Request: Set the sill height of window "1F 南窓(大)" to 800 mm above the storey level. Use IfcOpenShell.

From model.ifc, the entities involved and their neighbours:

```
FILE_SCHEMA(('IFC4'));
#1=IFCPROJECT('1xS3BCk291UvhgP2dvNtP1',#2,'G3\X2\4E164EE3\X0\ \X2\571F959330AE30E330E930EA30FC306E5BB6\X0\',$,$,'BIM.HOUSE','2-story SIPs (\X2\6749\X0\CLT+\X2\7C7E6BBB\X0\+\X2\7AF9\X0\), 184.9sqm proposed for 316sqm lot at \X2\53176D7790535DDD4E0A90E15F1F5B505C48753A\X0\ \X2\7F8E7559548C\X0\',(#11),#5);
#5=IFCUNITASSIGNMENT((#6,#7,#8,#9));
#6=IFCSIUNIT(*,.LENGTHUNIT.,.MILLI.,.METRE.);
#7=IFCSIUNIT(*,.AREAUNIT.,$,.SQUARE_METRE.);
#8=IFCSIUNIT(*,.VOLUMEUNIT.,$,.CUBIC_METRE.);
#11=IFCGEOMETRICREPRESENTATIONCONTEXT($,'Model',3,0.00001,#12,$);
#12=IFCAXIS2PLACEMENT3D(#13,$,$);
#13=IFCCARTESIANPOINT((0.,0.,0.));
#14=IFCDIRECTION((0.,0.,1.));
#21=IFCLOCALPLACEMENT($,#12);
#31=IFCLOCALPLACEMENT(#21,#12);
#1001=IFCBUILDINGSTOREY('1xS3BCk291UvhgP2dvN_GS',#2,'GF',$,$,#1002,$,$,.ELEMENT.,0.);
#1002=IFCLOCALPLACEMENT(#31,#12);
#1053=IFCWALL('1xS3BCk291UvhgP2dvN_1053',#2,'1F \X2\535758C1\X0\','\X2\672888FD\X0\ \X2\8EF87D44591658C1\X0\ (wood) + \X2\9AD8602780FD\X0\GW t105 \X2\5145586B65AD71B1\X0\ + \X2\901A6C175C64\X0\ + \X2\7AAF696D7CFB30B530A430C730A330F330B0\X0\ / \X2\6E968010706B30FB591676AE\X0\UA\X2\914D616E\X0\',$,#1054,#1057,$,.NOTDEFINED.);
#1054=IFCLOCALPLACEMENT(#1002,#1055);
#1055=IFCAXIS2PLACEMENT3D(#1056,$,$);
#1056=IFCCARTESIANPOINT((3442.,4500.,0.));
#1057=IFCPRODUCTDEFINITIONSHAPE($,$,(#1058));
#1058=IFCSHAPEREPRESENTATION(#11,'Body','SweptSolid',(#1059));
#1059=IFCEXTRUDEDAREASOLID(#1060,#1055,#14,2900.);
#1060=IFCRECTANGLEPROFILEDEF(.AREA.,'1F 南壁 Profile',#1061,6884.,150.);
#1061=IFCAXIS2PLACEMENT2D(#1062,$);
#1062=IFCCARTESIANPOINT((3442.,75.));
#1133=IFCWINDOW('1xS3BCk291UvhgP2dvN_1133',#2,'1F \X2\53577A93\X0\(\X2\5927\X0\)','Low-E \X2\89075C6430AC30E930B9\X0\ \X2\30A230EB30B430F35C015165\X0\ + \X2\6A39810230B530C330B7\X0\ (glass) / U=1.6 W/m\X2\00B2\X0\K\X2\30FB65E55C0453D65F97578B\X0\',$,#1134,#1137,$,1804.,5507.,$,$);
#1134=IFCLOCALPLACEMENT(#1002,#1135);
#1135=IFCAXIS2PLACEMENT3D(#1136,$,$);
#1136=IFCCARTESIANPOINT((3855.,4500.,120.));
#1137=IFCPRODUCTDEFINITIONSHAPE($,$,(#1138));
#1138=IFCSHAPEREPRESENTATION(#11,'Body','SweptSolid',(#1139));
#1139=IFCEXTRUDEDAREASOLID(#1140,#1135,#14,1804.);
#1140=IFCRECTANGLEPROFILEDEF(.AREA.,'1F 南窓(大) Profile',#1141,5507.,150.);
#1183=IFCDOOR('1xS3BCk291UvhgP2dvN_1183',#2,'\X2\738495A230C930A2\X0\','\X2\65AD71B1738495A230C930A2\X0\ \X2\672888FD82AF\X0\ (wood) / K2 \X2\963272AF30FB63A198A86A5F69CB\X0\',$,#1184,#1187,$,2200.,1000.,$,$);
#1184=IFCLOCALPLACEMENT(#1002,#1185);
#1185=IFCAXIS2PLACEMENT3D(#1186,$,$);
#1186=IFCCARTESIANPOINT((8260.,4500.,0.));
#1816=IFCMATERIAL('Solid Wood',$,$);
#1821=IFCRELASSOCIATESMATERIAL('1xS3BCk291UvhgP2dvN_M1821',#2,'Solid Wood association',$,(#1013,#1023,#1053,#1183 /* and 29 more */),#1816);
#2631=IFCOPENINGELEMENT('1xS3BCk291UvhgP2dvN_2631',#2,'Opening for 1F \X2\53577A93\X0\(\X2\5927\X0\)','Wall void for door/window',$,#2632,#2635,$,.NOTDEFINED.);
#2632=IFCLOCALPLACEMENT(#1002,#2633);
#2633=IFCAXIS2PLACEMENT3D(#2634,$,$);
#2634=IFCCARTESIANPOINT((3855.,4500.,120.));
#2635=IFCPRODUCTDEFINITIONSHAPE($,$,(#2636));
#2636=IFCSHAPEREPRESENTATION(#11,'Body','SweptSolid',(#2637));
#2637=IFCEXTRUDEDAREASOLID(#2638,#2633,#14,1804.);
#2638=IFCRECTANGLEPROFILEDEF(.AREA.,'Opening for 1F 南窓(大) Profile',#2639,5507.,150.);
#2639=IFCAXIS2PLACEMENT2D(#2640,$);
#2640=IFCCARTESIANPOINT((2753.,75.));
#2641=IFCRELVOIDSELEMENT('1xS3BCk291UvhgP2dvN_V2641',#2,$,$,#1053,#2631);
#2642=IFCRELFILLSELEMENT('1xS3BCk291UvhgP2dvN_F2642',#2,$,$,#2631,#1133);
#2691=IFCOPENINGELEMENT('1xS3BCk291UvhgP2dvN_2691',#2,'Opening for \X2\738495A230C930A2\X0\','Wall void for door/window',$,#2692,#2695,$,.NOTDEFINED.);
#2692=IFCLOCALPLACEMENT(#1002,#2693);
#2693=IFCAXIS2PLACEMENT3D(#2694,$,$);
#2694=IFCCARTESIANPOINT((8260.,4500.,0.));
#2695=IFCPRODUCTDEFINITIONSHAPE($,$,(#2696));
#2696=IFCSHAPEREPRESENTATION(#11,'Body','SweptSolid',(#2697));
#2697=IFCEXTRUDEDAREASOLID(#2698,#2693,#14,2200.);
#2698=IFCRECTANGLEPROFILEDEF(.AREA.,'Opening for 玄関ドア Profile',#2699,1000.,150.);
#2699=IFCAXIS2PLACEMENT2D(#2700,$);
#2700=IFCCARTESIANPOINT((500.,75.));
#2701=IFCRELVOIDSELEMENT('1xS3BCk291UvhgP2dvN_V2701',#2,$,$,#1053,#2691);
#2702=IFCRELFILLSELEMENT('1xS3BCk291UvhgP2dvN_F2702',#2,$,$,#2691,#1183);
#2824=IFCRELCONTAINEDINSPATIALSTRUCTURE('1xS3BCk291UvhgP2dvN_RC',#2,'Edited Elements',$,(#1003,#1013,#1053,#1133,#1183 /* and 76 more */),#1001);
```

```python
import numpy as np
import ifcopenshell
import ifcopenshell.api.geometry
import ifcopenshell.geom
import ifcopenshell.util.element
import ifcopenshell.util.placement
import ifcopenshell.util.shape
import ifcopenshell.util.unit

model = ifcopenshell.open("model.ifc")
unit_scale = ifcopenshell.util.unit.calculate_unit_scale(model)

window = model.by_id(1133)
opening = window.FillsVoids[0].RelatingOpeningElement
storey = ifcopenshell.util.element.get_container(window, ifc_class="IfcBuildingStorey")
level = ifcopenshell.util.placement.get_local_placement(storey.ObjectPlacement)[2, 3]

# The opening's origin need not be at the sill, so measure its lowest point.
shape = ifcopenshell.geom.create_shape(ifcopenshell.geom.settings(), opening)
bottom = ifcopenshell.util.shape.get_shape_bottom_elevation(shape, shape.geometry) / unit_scale
dz = level + 0.8 / unit_scale - bottom

shift = np.array([0.0, 0.0, dz])
# The window is not placed relative to its opening, so move both.
for product in (opening, window):
    matrix = ifcopenshell.util.placement.get_local_placement(product.ObjectPlacement)
    matrix[:3, 3] += shift
    ifcopenshell.api.geometry.edit_object_placement(model, product=product, matrix=matrix, is_si=False)

print(f"moved by {dz * unit_scale:+.3f} m")

model.write("model-out.ifc")
```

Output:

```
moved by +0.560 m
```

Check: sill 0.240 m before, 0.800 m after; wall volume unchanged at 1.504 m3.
